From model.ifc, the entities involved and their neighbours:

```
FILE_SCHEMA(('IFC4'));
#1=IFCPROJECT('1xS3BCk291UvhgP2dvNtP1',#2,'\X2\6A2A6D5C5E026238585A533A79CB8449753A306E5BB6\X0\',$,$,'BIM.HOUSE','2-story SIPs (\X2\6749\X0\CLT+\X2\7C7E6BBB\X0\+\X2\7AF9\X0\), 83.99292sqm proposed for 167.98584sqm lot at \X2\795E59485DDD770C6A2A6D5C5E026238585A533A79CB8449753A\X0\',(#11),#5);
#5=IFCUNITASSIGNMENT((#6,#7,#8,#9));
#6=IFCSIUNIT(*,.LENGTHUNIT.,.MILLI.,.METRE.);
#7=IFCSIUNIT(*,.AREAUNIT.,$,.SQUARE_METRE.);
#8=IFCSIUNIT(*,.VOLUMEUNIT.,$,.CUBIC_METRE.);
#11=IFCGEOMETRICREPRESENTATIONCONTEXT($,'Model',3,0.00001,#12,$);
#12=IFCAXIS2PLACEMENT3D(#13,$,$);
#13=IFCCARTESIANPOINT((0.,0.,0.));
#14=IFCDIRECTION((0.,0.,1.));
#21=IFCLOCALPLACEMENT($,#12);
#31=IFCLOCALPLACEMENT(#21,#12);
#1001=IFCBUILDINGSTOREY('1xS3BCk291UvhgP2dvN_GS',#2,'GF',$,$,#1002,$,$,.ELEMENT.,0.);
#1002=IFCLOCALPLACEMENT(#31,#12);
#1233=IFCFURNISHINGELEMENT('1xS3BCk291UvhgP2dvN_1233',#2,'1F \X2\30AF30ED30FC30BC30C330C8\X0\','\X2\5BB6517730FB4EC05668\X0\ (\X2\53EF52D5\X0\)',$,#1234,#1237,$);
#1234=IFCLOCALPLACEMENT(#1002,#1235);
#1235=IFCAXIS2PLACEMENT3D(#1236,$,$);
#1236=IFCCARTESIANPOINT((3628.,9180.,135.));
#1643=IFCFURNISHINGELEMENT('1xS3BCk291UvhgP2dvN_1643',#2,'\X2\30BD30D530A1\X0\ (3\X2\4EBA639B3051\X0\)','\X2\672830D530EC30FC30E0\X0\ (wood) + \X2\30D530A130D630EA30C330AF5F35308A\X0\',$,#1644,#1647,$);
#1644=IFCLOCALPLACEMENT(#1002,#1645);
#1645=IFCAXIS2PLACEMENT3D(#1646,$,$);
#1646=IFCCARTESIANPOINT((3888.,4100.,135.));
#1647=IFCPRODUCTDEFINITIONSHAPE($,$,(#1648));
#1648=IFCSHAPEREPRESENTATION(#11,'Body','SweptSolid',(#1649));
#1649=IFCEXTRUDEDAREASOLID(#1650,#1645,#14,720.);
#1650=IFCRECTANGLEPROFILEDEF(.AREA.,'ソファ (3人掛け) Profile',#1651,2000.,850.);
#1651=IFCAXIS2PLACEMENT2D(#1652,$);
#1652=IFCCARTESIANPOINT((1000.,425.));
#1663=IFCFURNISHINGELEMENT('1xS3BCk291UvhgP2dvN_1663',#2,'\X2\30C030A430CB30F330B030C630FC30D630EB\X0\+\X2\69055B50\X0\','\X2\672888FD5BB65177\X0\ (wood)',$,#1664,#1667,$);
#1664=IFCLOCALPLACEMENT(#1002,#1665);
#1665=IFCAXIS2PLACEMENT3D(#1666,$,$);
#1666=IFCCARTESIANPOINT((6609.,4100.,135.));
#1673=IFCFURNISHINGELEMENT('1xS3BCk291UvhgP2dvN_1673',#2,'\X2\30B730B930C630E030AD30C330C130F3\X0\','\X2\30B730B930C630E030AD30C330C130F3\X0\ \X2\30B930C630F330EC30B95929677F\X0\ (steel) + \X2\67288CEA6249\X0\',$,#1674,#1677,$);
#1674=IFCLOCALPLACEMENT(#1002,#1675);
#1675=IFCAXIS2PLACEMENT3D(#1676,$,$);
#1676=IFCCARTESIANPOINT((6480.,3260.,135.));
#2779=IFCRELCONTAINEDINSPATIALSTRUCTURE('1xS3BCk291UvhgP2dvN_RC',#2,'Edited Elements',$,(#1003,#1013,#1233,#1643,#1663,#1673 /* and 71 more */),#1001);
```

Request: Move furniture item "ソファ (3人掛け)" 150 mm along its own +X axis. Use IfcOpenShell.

```python
import ifcopenshell
import ifcopenshell.api.geometry
import ifcopenshell.util.placement
import ifcopenshell.util.unit

model = ifcopenshell.open("model.ifc")
unit_scale = ifcopenshell.util.unit.calculate_unit_scale(model)

item = model.by_guid("1xS3BCk291UvhgP2dvN_1643")
matrix = ifcopenshell.util.placement.get_local_placement(item.ObjectPlacement)
matrix[:3, 3] += matrix[:3, 0] * 0.15 / unit_scale
ifcopenshell.api.geometry.edit_object_placement(model, product=item, matrix=matrix, is_si=False)

print(ifcopenshell.util.placement.get_local_placement(item.ObjectPlacement).round(3) + 0.0)

model.write("model-out.ifc")
```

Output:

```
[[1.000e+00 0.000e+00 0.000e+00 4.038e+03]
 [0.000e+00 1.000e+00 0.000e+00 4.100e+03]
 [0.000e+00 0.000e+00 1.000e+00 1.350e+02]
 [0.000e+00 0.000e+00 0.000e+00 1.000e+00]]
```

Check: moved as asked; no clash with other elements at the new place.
